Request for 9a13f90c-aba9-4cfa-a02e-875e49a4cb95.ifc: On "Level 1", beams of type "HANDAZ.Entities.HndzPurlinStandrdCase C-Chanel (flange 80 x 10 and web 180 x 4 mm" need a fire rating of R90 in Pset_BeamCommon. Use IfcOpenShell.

First a look at what the model holds.

```python
import ifcopenshell
import ifcopenshell.util.element

model = ifcopenshell.open("9a13f90c-aba9-4cfa-a02e-875e49a4cb95.ifc")
print(model.schema)
storey = next(s for s in model.by_type("IfcBuildingStorey") if s.Name == "Level 1")
beams = [e for e in ifcopenshell.util.element.get_decomposition(storey) if e.is_a("IfcBeam")]
seen = {}
for e in beams:
    element_type = ifcopenshell.util.element.get_type(e)
    key = (element_type.Name if element_type != e and element_type else None, ifcopenshell.util.element.get_pset(e, "Pset_BeamCommon", "FireRating"))
    seen[key] = seen.get(key, 0) + 1
for (name, value), count in sorted(seen.items(), key=str):
    print(count, "x", name, "|", value)
```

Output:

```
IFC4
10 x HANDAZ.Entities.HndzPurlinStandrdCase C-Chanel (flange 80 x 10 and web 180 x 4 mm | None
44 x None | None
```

```python
import ifcopenshell
import ifcopenshell.api.pset
import ifcopenshell.util.element

model = ifcopenshell.open("9a13f90c-aba9-4cfa-a02e-875e49a4cb95.ifc")

storey = next(s for s in model.by_type("IfcBuildingStorey") if s.Name == "Level 1")
beams = [e for e in ifcopenshell.util.element.get_decomposition(storey) if e.is_a("IfcBeam")]

count = 0
for e in beams:
    element_type = ifcopenshell.util.element.get_type(e)
    if element_type in (None, e) or element_type.Name != "HANDAZ.Entities.HndzPurlinStandrdCase C-Chanel (flange 80 x 10 and web 180 x 4 mm":
        continue
    # add_pset returns the element's existing set when there is one.
    pset = ifcopenshell.api.pset.add_pset(model, product=e, name="Pset_BeamCommon")
    ifcopenshell.api.pset.edit_pset(model, pset=pset, properties={"FireRating": "R90"})
    count += 1

print(count, "beams updated")

model.write("9a13f90c-aba9-4cfa-a02e-875e49a4cb95_rev.ifc")
```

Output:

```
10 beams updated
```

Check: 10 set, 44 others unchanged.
